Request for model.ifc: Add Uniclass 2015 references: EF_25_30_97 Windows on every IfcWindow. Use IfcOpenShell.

First a look at what the model holds.

```python
import ifcopenshell

model = ifcopenshell.open("model.ifc")
print(model.schema)
print("classifications:", [c.Name for c in model.by_type("IfcClassification")])
for ifc_class in ("IfcDoor", "IfcRoof", "IfcStair", "IfcWall", "IfcWindow"):
    print(ifc_class, len(model.by_type(ifc_class)))
```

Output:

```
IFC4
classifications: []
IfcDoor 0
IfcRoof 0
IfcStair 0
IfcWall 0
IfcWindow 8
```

```python
import ifcopenshell
import ifcopenshell.api.classification

model = ifcopenshell.open("model.ifc")

system = ifcopenshell.api.classification.add_classification(model, classification="Uniclass 2015")

codes = {
    "IfcWindow": ("EF_25_30_97", "Windows"),
}
for ifc_class, (code, name) in codes.items():
    products = model.by_type(ifc_class)
    ifcopenshell.api.classification.add_reference(
        model, products=products, classification=system, identification=code, name=name
    )
    print(code, len(products))

model.write("model_edited.ifc")
```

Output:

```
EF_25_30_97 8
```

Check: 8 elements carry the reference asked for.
